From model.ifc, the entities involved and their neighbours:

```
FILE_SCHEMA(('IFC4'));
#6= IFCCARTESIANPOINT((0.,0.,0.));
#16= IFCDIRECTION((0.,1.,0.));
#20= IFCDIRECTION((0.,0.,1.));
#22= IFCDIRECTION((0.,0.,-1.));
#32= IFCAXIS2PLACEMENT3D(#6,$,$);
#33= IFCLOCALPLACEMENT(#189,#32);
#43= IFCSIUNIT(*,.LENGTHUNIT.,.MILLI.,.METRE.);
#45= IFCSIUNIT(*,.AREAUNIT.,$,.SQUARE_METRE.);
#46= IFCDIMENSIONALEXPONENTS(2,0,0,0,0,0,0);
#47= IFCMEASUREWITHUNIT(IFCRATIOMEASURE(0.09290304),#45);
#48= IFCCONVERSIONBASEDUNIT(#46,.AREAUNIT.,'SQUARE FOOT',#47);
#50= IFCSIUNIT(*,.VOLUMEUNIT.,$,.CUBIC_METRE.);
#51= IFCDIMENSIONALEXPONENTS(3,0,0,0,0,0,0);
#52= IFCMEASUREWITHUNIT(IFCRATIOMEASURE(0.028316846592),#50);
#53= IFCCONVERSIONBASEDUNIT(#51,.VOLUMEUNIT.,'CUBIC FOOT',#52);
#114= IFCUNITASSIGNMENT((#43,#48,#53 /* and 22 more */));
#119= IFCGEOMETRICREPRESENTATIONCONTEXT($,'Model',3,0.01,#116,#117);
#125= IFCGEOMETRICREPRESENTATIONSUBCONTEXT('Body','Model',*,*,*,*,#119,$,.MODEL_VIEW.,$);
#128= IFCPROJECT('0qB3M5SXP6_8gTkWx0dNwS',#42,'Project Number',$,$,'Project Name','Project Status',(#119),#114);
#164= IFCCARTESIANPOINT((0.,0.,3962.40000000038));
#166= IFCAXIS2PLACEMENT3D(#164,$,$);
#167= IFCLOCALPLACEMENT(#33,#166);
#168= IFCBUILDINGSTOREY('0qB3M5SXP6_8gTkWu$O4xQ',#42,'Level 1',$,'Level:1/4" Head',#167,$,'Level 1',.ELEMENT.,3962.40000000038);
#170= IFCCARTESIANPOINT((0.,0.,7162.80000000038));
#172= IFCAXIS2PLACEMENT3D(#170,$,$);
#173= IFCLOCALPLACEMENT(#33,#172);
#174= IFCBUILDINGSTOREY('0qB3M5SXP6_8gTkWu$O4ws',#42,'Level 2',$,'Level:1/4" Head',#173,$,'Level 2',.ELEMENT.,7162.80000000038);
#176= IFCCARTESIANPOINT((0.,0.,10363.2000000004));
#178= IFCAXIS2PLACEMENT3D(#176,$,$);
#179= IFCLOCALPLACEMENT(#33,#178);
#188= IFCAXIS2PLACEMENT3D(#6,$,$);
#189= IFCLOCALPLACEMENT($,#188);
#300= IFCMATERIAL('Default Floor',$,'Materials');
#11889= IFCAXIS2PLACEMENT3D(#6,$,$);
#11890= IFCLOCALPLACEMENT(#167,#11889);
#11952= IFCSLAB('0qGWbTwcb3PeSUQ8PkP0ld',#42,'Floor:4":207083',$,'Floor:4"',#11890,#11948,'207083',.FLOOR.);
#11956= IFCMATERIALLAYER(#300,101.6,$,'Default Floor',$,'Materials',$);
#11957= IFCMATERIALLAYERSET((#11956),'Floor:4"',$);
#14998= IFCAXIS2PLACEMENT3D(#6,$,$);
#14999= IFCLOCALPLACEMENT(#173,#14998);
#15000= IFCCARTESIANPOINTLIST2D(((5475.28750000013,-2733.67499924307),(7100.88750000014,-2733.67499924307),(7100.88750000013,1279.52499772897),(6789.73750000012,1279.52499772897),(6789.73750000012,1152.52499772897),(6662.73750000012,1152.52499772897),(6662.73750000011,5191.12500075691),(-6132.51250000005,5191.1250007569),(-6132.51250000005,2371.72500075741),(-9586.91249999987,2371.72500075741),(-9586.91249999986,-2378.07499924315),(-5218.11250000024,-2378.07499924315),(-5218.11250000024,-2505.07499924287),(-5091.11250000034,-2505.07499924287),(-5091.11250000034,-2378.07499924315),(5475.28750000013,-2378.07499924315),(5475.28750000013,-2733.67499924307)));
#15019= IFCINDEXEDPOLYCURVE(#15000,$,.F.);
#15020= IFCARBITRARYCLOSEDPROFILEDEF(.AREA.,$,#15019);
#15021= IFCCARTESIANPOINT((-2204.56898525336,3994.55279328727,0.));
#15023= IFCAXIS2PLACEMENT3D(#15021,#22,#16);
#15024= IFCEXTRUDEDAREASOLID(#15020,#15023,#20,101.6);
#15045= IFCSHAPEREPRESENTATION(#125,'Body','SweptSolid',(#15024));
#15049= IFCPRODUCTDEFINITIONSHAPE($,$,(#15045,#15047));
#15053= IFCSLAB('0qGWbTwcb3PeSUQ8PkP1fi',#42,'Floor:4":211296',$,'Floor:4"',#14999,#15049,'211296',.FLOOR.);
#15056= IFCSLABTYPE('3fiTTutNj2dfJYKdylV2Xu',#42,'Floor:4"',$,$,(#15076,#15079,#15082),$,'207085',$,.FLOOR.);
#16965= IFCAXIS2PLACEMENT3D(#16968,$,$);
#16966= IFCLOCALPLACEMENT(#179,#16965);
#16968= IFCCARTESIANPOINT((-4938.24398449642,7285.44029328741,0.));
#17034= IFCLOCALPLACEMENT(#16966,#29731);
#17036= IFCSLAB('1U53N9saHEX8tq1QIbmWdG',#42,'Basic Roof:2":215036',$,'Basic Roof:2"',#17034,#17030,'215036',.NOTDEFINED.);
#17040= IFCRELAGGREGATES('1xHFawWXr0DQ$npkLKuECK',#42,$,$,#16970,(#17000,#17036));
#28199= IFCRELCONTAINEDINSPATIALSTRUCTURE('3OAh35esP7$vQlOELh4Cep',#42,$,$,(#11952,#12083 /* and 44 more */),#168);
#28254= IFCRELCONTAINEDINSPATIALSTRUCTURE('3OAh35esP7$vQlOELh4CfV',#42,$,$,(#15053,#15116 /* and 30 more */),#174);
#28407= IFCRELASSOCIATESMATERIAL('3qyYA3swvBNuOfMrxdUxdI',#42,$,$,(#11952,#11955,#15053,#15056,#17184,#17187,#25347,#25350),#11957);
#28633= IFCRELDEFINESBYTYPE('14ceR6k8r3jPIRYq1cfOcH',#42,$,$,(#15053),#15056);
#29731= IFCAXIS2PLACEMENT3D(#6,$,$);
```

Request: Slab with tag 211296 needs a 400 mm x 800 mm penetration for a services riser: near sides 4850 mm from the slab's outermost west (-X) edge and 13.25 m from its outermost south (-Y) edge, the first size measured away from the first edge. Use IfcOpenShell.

```python
import numpy as np
import ifcopenshell
import ifcopenshell.api.feature
import ifcopenshell.api.geometry
import ifcopenshell.api.root
import ifcopenshell.geom
import ifcopenshell.util.placement
import ifcopenshell.util.representation
import ifcopenshell.util.shape
import ifcopenshell.util.unit

model = ifcopenshell.open("model.ifc")
unit_scale = ifcopenshell.util.unit.calculate_unit_scale(model)
settings = ifcopenshell.geom.settings()


def volume(element):
    """Net volume in cubic metres, openings subtracted."""
    shape = ifcopenshell.geom.create_shape(settings, element)
    return ifcopenshell.util.shape.get_volume(shape.geometry)


slab = model.by_guid("0qGWbTwcb3PeSUQ8PkP1fi")
before = volume(slab)

# Extent in the slab's own axes, in metres. The edges named are its -X and -Y sides.
slab_shape = ifcopenshell.geom.create_shape(settings, slab)
vertices = ifcopenshell.util.shape.get_vertices(slab_shape.geometry)
x_min, y_min, bottom = vertices.min(axis=0)
top = vertices[:, 2].max()

opening = ifcopenshell.api.root.create_entity(model, ifc_class="IfcOpeningElement", name="Services riser opening", predefined_type="OPENING")
context = ifcopenshell.util.representation.get_context(model, "Model", "Body", "MODEL_VIEW")
width, depth = 0.4, 0.8
outline = [(0.0, 0.0), (width, 0.0), (width, depth), (0.0, depth), (0.0, 0.0)]
# Overshoot both faces by 50 mm so the cut is clean.
shape = ifcopenshell.api.geometry.add_slab_representation(
    model, context=context, depth=top - bottom + 0.1, polyline=outline
)
ifcopenshell.api.geometry.assign_representation(model, product=opening, representation=shape)

matrix = ifcopenshell.util.placement.get_local_placement(slab.ObjectPlacement)
matrix[:, 3] = matrix @ np.append(np.array([x_min + 4.85, y_min + 13.25, bottom - 0.05]) / unit_scale, 1.0)
ifcopenshell.api.geometry.edit_object_placement(model, product=opening, matrix=matrix, is_si=False)
ifcopenshell.api.feature.add_feature(model, feature=opening, element=slab)

after = volume(slab)

print(f"slab volume {before:.3f} -> {after:.3f} m3")

model.write("model-out.ifc")
```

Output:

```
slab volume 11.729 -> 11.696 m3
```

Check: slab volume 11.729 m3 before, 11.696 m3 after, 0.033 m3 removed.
